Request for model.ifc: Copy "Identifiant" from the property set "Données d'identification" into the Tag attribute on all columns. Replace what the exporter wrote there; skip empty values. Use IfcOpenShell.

First a look at what the model holds.

```python
import ifcopenshell
import ifcopenshell.util.element

model = ifcopenshell.open("model.ifc")
print(model.schema)
columns = model.by_type("IfcColumn")
print(len(columns), "columns")
for e in columns[:8]:
    source = ifcopenshell.util.element.get_pset(e, "Données d'identification", "Identifiant")
    target = e.Tag
    print(e.id(), repr(source), repr(target), sep=" | ")
```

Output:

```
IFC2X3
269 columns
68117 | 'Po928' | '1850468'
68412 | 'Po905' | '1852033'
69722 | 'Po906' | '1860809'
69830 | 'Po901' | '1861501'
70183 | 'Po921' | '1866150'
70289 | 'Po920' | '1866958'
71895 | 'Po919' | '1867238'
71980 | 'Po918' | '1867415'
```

```python
import ifcopenshell
import ifcopenshell.util.element

model = ifcopenshell.open("model.ifc")

count = 0
for e in model.by_type("IfcColumn"):
    value = ifcopenshell.util.element.get_pset(e, "Données d'identification", "Identifiant")
    current = e.Tag
    if not value or not value.strip() or current == value:
        continue
    e.Tag = value
    count += 1

print(count, "columns updated")

model.write("model_rev.ifc")
```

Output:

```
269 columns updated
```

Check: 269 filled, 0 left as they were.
